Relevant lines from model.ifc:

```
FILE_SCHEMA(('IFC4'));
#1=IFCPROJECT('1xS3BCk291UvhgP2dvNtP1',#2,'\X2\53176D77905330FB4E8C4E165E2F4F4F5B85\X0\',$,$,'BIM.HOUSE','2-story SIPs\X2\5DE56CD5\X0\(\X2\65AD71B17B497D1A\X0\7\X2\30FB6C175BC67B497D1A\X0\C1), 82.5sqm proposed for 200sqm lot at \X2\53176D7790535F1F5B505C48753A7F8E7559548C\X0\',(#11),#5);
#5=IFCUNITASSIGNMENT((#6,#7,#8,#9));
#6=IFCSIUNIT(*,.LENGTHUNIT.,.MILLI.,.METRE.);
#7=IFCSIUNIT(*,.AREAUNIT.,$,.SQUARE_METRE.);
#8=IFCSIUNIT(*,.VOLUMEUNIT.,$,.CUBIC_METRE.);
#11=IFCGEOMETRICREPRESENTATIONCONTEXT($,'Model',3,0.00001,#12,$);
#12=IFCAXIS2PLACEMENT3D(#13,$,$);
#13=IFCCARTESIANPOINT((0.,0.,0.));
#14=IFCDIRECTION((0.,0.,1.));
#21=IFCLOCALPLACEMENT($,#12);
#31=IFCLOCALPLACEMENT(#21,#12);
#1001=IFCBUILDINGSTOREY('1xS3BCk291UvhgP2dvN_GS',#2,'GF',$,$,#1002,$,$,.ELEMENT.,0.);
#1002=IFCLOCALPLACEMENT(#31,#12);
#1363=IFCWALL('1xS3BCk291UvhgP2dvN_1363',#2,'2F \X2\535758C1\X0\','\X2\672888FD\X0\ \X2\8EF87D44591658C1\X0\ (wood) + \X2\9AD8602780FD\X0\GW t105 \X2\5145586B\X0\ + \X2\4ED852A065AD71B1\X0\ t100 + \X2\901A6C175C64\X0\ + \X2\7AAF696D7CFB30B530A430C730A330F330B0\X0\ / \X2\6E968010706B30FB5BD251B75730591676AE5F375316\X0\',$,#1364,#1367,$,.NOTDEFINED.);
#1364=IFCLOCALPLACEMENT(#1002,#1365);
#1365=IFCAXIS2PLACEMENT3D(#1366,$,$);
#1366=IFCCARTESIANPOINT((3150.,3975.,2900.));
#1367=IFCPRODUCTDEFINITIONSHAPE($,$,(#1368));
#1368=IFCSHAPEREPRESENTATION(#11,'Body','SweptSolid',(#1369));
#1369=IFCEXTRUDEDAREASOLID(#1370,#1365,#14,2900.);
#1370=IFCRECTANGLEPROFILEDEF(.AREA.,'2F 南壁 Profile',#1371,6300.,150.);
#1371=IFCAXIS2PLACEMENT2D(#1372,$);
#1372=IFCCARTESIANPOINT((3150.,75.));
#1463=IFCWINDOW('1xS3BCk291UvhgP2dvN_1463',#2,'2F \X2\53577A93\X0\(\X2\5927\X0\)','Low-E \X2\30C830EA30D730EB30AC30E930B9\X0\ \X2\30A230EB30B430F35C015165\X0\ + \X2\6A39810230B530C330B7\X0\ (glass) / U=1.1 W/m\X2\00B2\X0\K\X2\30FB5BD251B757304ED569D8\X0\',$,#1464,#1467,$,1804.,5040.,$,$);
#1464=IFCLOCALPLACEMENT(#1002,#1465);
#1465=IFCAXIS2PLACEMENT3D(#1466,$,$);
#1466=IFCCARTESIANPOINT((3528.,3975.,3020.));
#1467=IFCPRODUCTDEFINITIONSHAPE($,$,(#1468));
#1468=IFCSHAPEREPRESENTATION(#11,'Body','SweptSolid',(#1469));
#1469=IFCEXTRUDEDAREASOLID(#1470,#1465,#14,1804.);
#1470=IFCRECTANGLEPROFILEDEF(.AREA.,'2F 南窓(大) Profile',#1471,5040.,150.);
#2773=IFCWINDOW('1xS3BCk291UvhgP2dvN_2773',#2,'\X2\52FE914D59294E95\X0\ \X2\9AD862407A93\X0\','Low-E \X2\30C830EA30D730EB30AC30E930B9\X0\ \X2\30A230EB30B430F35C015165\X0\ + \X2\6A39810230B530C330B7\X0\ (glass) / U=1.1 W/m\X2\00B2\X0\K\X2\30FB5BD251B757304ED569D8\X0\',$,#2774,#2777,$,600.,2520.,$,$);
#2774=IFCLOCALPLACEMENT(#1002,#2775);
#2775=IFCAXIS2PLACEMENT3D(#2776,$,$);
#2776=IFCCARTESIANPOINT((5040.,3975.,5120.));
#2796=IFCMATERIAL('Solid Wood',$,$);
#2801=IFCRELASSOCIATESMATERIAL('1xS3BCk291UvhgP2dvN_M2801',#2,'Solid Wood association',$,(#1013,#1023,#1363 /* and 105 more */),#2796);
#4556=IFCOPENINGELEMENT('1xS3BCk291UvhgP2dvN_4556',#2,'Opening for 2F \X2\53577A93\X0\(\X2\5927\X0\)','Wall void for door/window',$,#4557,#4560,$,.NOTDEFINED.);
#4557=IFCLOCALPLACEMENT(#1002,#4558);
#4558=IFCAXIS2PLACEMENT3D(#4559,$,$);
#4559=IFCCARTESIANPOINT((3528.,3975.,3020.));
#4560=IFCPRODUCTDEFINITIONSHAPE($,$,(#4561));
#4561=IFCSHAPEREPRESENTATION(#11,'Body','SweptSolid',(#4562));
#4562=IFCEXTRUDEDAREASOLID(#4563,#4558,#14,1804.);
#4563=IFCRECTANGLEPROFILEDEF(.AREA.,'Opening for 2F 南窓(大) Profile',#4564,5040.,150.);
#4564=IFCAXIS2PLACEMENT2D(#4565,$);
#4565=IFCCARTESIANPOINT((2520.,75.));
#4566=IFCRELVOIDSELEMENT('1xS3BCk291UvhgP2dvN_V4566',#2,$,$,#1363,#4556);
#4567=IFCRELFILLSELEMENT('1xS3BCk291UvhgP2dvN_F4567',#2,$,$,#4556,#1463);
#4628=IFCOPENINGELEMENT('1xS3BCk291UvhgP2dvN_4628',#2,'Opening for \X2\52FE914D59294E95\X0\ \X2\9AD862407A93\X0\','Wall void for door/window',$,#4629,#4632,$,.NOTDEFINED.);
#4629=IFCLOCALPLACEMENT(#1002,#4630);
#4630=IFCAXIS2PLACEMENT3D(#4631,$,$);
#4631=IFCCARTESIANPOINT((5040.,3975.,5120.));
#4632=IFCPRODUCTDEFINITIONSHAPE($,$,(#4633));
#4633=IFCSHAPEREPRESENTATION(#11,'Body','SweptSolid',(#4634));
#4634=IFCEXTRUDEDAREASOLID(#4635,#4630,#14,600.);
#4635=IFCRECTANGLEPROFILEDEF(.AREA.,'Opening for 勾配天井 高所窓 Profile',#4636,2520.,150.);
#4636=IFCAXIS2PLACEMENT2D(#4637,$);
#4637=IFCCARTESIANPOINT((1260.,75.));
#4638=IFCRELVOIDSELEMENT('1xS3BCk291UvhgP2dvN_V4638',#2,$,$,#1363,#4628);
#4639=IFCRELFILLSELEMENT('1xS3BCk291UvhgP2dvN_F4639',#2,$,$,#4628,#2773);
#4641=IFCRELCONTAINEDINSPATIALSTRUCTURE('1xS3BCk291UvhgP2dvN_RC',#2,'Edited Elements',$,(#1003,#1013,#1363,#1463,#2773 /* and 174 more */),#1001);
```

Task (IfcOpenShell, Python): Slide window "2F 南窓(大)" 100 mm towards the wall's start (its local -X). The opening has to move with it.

```python
import ifcopenshell
import ifcopenshell.api.geometry
import ifcopenshell.util.placement

model = ifcopenshell.open("model.ifc")

window = model.by_guid("1xS3BCk291UvhgP2dvN_1463")
opening = window.FillsVoids[0].RelatingOpeningElement
wall = opening.VoidsElements[0].RelatingBuildingElement

wall_matrix = ifcopenshell.util.placement.get_local_placement(wall.ObjectPlacement)
shift = wall_matrix[:3, 0] * -100.0
before = ifcopenshell.util.placement.get_local_placement(window.ObjectPlacement)[:3, 3].copy()

# The window is not placed relative to its opening, so move both.
for product in (opening, window):
    matrix = ifcopenshell.util.placement.get_local_placement(product.ObjectPlacement)
    matrix[:3, 3] += shift
    ifcopenshell.api.geometry.edit_object_placement(model, product=product, matrix=matrix, is_si=False)

after = ifcopenshell.util.placement.get_local_placement(window.ObjectPlacement)[:3, 3]
print("window moved by", (after - before).round(3) + 0.0)

model.write("model_updated.ifc")
```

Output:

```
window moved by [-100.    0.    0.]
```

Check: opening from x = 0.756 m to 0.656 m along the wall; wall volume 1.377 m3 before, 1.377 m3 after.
